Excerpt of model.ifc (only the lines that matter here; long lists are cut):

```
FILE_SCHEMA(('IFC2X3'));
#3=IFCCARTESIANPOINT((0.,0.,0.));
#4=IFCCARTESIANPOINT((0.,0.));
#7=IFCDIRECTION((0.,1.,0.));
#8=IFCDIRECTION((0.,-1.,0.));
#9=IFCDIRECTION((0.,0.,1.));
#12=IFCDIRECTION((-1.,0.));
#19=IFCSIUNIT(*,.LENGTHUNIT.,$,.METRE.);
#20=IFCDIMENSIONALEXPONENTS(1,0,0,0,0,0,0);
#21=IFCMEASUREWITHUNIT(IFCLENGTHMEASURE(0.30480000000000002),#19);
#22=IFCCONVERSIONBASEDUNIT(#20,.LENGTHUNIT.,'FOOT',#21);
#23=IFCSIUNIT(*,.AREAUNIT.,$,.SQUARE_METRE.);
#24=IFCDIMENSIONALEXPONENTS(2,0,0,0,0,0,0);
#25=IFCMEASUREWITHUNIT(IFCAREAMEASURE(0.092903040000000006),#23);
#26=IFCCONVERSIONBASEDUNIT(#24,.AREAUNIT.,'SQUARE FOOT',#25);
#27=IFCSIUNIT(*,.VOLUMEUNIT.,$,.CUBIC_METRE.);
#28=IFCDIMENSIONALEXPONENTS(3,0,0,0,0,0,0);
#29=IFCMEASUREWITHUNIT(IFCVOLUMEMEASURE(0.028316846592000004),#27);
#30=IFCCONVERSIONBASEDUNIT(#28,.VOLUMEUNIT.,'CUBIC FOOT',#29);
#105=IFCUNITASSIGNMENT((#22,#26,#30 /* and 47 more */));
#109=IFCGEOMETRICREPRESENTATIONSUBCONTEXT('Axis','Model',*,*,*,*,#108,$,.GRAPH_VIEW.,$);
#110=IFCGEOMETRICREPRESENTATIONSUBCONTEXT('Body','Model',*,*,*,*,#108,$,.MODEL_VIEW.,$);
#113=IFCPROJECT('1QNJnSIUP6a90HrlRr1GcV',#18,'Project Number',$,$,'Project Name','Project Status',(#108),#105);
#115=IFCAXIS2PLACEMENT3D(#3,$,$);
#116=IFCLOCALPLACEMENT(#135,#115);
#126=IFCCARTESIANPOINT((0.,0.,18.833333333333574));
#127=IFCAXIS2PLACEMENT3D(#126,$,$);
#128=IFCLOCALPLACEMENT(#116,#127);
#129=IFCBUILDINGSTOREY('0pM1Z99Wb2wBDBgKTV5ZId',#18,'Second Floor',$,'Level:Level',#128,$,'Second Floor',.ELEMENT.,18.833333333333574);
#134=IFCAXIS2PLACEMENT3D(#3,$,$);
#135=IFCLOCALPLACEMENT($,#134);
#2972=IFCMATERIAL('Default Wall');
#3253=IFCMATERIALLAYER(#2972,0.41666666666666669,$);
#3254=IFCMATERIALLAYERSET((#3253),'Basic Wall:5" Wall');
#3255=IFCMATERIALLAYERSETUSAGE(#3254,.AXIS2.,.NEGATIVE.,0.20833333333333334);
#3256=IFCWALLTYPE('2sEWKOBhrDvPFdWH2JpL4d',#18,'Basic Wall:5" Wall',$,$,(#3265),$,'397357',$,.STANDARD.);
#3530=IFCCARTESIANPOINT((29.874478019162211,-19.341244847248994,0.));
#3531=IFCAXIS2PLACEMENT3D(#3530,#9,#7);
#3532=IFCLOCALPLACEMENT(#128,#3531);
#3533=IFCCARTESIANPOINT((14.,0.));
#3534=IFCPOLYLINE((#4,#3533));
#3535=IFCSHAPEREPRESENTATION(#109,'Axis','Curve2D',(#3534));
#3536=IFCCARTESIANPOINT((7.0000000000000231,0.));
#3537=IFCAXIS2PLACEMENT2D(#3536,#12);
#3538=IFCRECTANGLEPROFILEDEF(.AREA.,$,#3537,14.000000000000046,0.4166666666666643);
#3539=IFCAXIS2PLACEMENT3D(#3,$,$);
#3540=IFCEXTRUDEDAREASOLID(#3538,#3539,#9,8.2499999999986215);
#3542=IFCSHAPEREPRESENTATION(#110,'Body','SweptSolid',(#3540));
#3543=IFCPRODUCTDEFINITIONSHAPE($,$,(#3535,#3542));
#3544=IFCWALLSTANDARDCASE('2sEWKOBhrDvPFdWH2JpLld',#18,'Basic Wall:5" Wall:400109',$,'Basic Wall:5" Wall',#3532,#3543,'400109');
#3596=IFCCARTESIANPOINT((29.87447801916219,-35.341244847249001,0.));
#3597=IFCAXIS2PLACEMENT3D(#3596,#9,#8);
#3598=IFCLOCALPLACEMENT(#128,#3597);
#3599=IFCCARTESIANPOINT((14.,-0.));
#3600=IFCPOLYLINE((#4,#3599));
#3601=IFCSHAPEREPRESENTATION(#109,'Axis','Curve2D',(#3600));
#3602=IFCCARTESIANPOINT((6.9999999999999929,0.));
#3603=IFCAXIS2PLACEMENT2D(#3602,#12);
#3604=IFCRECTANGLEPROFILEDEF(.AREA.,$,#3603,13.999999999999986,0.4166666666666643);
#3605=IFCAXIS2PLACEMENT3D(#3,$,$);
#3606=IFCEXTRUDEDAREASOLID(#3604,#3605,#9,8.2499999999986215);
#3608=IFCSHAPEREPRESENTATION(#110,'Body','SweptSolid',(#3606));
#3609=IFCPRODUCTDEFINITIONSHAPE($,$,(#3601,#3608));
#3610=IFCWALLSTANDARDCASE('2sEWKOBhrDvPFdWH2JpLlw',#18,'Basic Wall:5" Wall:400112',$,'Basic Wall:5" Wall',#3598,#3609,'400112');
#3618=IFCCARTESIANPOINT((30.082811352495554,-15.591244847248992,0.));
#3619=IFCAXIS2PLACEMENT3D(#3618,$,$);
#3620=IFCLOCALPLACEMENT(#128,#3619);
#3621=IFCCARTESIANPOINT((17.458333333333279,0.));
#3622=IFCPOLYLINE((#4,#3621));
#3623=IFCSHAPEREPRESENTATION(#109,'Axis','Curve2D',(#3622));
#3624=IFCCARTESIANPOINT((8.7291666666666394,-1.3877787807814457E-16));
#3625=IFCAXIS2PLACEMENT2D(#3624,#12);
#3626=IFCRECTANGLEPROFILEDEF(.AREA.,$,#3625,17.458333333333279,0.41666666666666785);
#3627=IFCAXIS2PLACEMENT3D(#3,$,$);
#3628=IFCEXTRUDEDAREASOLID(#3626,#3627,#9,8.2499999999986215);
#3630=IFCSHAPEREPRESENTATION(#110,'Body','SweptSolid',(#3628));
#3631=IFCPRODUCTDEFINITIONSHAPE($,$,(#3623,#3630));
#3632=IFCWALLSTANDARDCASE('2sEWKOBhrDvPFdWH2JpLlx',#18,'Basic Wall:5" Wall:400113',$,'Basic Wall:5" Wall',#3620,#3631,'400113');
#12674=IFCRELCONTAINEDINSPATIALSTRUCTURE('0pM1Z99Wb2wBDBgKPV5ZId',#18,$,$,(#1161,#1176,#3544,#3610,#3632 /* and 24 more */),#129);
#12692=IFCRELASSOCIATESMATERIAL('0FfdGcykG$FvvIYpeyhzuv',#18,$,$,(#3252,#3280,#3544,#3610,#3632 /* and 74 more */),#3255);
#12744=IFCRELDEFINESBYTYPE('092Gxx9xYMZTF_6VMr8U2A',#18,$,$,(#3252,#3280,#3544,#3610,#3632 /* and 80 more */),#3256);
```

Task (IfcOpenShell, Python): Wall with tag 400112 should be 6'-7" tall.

```python
import ifcopenshell
import ifcopenshell.geom
import ifcopenshell.util.representation
import ifcopenshell.util.shape
import ifcopenshell.util.unit

model = ifcopenshell.open("model.ifc")
unit_scale = ifcopenshell.util.unit.calculate_unit_scale(model)
settings = ifcopenshell.geom.settings()


def volume(element):
    """Net volume in cubic metres, openings subtracted."""
    shape = ifcopenshell.geom.create_shape(settings, element)
    return ifcopenshell.util.shape.get_volume(shape.geometry)


wall = model.by_guid("2sEWKOBhrDvPFdWH2JpLlw")
before = volume(wall)

body = ifcopenshell.util.representation.get_representation(wall, "Model", "Body")
solid = body.Items[0]
old_height = solid.Depth
solid.Depth = 79 * 0.0254 / unit_scale
after = volume(wall)

print(f"height {old_height:g} -> {solid.Depth:g}, volume {before:.3f} -> {after:.3f} m3")

model.write("model_rev.ifc")
```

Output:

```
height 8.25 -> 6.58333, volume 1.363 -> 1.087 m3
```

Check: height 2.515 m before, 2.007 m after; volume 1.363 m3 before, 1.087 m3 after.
